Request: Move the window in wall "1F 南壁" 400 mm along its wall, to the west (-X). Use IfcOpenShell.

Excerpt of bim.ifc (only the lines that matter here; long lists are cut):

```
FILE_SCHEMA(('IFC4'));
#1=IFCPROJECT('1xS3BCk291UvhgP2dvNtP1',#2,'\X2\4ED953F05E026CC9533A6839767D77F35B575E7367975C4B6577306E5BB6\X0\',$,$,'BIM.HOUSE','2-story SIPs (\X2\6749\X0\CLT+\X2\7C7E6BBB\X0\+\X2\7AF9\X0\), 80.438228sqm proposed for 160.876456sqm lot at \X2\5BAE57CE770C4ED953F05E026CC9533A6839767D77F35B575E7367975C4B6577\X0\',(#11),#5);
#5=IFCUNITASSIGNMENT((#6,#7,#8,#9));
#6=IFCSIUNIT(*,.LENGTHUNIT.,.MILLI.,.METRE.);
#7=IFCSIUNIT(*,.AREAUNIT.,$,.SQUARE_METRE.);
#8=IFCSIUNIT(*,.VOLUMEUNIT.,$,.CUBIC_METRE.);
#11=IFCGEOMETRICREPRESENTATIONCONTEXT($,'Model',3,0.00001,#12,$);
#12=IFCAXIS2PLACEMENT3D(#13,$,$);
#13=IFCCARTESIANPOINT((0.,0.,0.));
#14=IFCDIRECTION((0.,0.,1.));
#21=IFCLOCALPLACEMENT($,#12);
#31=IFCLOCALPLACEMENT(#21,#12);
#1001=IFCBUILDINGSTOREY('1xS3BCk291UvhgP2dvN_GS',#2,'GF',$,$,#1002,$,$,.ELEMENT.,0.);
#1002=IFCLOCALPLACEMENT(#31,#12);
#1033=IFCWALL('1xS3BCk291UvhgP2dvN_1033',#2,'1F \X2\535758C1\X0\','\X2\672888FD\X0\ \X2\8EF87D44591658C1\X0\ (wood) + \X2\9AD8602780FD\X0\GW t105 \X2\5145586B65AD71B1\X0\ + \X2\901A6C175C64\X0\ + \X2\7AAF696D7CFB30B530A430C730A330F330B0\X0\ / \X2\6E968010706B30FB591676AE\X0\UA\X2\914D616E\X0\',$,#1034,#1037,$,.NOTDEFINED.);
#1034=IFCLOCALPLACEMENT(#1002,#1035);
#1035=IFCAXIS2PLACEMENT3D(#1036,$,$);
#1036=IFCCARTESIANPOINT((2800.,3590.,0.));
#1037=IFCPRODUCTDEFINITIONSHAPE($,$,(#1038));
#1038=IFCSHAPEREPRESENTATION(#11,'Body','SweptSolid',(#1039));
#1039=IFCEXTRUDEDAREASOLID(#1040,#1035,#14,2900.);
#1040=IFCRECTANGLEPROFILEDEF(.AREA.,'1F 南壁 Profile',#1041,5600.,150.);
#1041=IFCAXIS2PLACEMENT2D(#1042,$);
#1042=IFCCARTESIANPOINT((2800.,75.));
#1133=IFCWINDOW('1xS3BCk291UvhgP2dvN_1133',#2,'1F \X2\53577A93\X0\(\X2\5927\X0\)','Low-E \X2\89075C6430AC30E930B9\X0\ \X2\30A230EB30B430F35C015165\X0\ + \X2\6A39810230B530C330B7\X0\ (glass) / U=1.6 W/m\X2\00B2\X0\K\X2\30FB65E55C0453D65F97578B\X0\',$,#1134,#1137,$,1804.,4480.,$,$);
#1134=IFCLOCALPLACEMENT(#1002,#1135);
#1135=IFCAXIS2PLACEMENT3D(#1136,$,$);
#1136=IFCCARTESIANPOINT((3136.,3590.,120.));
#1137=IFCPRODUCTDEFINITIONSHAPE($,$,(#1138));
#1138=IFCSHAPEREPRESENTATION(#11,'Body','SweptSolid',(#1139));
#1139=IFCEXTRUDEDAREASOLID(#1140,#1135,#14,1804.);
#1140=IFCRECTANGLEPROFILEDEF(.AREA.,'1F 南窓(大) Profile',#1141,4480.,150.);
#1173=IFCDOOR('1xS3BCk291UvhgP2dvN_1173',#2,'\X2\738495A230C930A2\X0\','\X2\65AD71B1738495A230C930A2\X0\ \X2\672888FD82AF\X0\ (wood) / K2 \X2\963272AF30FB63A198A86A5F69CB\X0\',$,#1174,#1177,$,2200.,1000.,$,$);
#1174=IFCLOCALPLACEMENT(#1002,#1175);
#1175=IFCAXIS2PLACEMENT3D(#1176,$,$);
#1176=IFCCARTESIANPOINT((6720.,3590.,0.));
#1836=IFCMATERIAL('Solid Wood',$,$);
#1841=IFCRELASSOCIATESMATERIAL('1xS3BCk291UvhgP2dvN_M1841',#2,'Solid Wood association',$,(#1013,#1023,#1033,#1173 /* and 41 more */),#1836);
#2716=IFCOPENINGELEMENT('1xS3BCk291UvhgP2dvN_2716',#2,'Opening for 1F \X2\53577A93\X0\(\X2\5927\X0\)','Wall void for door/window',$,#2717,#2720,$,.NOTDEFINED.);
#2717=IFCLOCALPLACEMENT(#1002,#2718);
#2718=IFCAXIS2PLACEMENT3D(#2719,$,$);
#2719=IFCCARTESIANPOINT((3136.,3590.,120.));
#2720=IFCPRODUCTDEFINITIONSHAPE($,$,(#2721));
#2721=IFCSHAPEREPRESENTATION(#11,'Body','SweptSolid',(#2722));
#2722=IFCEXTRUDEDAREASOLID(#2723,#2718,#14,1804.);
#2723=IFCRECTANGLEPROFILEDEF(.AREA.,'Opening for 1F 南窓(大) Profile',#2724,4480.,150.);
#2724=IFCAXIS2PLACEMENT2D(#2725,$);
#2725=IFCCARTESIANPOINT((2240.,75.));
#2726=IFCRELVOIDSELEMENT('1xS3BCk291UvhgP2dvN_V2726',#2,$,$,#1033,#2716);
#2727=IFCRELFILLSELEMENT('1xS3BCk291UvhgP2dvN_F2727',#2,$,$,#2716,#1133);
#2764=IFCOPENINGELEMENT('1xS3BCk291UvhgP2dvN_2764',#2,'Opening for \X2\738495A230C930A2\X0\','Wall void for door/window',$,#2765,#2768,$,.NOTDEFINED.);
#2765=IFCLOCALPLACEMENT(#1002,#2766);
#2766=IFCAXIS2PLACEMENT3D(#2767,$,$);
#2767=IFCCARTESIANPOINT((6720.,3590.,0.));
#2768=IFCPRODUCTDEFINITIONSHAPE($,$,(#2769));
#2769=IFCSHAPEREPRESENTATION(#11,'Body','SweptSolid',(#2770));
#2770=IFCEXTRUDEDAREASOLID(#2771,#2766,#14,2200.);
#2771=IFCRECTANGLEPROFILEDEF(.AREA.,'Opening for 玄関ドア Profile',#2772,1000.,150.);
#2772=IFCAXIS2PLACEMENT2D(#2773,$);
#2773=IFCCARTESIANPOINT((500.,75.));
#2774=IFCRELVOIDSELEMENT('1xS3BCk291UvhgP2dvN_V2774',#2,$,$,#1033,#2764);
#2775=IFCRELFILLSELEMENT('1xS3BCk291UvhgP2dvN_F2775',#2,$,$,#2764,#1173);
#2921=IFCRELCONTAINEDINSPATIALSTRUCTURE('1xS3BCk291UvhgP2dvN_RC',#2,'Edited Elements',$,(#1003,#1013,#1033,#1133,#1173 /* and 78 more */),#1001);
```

```python
import ifcopenshell
import ifcopenshell.api.geometry
import ifcopenshell.util.placement

model = ifcopenshell.open("bim.ifc")

window = model.by_id(1133)
opening = window.FillsVoids[0].RelatingOpeningElement
wall = opening.VoidsElements[0].RelatingBuildingElement

wall_matrix = ifcopenshell.util.placement.get_local_placement(wall.ObjectPlacement)
shift = wall_matrix[:3, 0] * -400.0
before = ifcopenshell.util.placement.get_local_placement(window.ObjectPlacement)[:3, 3].copy()

# The window is not placed relative to its opening, so move both.
for product in (opening, window):
    matrix = ifcopenshell.util.placement.get_local_placement(product.ObjectPlacement)
    matrix[:3, 3] += shift
    ifcopenshell.api.geometry.edit_object_placement(model, product=product, matrix=matrix, is_si=False)

after = ifcopenshell.util.placement.get_local_placement(window.ObjectPlacement)[:3, 3]
print("window moved by", (after - before).round(3) + 0.0)

model.write("bim-out.ifc")
```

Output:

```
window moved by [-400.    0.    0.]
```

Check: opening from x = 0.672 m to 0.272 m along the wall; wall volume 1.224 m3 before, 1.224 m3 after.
